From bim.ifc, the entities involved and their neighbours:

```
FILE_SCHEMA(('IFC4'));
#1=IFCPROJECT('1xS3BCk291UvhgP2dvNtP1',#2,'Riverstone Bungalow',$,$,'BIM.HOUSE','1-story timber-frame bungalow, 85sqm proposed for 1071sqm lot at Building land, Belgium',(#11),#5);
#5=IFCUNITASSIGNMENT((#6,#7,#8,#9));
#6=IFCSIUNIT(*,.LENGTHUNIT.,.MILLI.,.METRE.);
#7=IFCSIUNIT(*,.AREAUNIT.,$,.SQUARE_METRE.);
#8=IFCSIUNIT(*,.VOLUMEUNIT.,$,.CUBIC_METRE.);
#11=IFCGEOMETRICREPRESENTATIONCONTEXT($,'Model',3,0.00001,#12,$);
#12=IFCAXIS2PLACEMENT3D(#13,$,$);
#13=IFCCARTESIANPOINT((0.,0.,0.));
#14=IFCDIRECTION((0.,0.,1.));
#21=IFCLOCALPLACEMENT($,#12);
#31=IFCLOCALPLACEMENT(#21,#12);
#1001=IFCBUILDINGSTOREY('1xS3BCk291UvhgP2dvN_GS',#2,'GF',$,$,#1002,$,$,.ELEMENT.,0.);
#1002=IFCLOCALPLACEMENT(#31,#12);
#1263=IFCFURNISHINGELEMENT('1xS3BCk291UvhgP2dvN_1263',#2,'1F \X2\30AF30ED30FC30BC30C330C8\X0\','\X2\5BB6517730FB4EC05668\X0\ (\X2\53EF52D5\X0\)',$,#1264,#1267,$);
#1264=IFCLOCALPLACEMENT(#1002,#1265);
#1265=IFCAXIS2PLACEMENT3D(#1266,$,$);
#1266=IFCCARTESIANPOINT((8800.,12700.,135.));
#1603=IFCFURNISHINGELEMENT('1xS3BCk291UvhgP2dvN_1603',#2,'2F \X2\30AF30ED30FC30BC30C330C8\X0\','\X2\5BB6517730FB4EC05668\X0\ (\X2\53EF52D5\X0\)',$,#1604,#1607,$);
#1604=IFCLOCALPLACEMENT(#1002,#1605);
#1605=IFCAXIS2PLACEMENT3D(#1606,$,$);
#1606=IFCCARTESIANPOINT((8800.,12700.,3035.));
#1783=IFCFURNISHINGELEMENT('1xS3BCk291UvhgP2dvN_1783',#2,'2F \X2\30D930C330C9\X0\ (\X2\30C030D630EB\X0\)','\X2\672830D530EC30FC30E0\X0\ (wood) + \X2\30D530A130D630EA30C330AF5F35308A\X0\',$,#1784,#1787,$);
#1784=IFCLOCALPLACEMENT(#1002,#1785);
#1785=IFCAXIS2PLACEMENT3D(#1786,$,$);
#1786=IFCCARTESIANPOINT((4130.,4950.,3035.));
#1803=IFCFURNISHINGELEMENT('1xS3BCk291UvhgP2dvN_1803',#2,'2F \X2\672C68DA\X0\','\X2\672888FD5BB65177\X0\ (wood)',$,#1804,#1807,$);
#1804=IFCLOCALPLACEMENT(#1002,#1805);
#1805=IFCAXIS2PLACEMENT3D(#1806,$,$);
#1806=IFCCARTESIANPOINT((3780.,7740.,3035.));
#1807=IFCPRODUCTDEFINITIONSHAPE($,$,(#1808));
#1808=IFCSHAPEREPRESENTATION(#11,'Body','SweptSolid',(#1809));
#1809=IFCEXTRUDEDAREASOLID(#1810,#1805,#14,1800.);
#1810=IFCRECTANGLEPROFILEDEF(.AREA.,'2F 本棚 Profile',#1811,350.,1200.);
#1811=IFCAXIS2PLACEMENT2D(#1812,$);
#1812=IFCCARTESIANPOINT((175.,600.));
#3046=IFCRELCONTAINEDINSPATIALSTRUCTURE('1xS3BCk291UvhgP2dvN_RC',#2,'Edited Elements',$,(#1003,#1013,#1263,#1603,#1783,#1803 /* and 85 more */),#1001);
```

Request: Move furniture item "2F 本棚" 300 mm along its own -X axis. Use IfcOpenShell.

```python
import ifcopenshell
import ifcopenshell.api.geometry
import ifcopenshell.util.placement
import ifcopenshell.util.unit

model = ifcopenshell.open("bim.ifc")
unit_scale = ifcopenshell.util.unit.calculate_unit_scale(model)

item = model.by_guid("1xS3BCk291UvhgP2dvN_1803")
matrix = ifcopenshell.util.placement.get_local_placement(item.ObjectPlacement)
matrix[:3, 3] -= matrix[:3, 0] * 0.3 / unit_scale
ifcopenshell.api.geometry.edit_object_placement(model, product=item, matrix=matrix, is_si=False)

print(ifcopenshell.util.placement.get_local_placement(item.ObjectPlacement).round(3) + 0.0)

model.write("bim_rev.ifc")
```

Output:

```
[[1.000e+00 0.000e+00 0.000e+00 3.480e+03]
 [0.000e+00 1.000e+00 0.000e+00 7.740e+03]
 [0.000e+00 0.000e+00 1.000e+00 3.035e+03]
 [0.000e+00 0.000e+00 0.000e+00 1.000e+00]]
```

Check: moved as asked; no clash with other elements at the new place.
